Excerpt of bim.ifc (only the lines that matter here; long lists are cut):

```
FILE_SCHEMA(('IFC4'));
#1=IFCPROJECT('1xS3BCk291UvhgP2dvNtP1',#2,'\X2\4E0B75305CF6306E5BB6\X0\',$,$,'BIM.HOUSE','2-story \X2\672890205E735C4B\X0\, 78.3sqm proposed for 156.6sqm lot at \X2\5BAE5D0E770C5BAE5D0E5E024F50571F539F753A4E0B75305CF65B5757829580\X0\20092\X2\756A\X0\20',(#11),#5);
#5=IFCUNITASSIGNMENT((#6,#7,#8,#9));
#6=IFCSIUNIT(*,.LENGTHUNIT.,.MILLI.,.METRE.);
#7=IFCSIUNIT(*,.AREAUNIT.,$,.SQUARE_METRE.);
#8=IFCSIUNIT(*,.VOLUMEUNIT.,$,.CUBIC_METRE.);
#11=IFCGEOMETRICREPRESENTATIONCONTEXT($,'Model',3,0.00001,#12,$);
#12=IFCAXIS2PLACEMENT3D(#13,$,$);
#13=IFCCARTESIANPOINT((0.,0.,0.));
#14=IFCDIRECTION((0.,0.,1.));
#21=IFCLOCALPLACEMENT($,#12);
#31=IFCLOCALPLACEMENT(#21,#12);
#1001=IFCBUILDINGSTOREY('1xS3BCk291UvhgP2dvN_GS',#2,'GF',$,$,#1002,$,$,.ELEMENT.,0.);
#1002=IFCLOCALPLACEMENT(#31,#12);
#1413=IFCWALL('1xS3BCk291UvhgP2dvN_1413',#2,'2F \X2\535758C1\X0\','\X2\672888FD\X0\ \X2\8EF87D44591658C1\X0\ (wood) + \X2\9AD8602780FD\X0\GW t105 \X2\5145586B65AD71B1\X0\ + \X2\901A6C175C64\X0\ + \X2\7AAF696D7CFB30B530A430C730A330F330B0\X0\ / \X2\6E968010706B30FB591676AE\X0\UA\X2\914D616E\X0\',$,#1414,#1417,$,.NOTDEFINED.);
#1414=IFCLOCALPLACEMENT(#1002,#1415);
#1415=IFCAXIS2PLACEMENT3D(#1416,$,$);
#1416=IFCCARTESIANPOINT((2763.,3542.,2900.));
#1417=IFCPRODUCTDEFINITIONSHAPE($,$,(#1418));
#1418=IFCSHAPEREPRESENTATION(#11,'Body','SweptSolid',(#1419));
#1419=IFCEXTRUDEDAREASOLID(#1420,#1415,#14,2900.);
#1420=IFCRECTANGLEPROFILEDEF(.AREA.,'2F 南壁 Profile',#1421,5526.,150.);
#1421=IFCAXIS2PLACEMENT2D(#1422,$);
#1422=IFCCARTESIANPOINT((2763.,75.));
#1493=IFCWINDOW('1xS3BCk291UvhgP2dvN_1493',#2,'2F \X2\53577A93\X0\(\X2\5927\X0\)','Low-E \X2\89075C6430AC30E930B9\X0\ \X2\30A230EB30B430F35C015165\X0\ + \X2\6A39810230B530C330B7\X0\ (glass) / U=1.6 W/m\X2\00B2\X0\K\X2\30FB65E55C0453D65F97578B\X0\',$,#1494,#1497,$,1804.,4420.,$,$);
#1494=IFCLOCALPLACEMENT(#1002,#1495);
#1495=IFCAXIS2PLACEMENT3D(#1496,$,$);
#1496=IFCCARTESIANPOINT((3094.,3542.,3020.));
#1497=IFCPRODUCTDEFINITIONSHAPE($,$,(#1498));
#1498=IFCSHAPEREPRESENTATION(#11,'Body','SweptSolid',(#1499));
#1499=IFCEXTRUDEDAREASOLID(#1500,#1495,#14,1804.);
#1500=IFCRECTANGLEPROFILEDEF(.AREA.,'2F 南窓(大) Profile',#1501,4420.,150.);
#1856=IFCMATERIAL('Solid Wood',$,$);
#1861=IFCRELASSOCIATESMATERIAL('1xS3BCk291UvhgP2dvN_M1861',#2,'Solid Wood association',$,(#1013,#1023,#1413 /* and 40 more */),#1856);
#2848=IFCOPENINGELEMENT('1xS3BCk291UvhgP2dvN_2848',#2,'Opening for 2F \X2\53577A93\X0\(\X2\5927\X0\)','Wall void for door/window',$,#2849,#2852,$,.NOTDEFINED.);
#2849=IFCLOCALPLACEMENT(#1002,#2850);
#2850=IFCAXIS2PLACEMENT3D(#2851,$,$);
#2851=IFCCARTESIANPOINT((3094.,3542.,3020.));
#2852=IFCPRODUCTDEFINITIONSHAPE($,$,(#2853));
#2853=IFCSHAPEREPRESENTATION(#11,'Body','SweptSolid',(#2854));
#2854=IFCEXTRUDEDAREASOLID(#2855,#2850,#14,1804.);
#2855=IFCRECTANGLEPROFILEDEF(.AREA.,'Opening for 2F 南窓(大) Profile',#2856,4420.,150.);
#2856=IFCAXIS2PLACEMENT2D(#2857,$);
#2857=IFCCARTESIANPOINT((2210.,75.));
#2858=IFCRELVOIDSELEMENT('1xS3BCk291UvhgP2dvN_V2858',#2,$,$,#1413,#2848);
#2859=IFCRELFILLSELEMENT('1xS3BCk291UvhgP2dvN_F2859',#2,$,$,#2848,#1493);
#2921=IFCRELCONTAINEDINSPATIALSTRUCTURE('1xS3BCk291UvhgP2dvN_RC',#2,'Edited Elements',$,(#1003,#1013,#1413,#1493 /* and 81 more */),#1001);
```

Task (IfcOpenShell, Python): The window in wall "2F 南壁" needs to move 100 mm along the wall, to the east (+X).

```python
import ifcopenshell
import ifcopenshell.api.geometry
import ifcopenshell.util.placement
import ifcopenshell.util.unit

model = ifcopenshell.open("bim.ifc")
unit_scale = ifcopenshell.util.unit.calculate_unit_scale(model)

window = model.by_id(1493)
opening = window.FillsVoids[0].RelatingOpeningElement
wall = opening.VoidsElements[0].RelatingBuildingElement

wall_matrix = ifcopenshell.util.placement.get_local_placement(wall.ObjectPlacement)
shift = wall_matrix[:3, 0] * 0.1 / unit_scale
before = ifcopenshell.util.placement.get_local_placement(window.ObjectPlacement)[:3, 3].copy()

# The window is not placed relative to its opening, so move both.
for product in (opening, window):
    matrix = ifcopenshell.util.placement.get_local_placement(product.ObjectPlacement)
    matrix[:3, 3] += shift
    ifcopenshell.api.geometry.edit_object_placement(model, product=product, matrix=matrix, is_si=False)

after = ifcopenshell.util.placement.get_local_placement(window.ObjectPlacement)[:3, 3]
print("window moved by", (after - before).round(3) + 0.0)

model.write("bim_updated.ifc")
```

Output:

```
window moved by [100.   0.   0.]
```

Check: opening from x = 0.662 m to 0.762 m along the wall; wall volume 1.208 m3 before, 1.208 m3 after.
